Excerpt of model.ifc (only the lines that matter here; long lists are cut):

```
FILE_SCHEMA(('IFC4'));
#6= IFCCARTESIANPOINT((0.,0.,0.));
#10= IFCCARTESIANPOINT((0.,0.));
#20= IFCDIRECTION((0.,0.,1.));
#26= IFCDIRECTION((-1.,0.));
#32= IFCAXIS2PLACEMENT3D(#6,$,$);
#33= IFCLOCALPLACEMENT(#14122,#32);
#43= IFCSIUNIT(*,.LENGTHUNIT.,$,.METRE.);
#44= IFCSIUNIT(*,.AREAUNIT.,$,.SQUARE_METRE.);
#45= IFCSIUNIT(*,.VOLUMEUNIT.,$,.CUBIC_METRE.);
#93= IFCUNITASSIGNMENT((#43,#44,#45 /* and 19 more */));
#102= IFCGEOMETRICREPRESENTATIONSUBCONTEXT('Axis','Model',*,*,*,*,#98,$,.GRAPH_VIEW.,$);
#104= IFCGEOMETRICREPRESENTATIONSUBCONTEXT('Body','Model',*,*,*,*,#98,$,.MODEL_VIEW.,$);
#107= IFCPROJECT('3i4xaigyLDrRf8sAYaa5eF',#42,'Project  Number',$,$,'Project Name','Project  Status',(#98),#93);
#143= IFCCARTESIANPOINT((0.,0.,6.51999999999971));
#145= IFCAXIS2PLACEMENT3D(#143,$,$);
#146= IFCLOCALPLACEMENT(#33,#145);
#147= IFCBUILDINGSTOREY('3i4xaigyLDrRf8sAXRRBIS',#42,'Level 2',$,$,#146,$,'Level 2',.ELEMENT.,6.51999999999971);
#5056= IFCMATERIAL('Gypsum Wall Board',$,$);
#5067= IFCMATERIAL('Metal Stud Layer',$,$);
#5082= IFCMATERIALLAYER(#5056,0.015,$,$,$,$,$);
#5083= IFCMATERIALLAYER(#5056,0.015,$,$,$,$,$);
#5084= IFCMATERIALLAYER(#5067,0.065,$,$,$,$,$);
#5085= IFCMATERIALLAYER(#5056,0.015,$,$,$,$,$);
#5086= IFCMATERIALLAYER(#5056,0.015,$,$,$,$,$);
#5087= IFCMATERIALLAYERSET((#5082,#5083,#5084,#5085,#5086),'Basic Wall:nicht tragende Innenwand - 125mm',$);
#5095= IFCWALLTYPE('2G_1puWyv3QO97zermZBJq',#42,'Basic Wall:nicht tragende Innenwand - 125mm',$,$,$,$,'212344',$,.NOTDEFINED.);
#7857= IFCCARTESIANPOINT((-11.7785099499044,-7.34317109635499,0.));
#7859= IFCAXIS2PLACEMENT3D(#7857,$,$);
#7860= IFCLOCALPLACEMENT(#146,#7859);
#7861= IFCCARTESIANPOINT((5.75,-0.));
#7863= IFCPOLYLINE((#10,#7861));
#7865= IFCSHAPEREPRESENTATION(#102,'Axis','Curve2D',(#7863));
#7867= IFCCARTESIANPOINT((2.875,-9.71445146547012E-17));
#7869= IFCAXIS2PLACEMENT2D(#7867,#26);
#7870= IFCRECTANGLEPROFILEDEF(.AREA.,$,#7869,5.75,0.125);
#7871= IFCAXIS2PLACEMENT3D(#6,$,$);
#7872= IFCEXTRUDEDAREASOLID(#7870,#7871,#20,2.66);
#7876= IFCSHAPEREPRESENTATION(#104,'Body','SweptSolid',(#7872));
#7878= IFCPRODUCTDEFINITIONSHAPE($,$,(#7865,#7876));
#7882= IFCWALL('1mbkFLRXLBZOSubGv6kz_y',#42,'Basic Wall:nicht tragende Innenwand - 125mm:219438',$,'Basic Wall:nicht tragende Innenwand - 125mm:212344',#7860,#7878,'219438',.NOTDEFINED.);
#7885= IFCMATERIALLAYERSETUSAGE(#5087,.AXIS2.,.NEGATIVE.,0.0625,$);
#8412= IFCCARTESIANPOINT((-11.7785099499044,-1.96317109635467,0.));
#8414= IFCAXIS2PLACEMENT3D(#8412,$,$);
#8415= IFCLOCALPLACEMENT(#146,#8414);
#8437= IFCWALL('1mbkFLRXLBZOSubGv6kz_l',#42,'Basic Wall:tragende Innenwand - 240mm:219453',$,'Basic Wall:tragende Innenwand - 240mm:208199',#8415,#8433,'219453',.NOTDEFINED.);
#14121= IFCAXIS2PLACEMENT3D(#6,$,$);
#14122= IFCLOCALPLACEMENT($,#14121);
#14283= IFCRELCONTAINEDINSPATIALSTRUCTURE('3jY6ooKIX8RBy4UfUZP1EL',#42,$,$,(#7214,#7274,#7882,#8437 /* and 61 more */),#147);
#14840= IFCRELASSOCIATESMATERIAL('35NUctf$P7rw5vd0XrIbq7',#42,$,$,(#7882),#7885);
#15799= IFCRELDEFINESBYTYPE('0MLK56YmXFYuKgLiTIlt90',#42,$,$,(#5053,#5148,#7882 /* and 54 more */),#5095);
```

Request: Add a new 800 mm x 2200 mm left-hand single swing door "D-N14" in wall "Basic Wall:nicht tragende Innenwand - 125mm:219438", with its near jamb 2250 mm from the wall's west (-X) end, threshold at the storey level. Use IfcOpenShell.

```python
import numpy as np
import ifcopenshell
import ifcopenshell.api.feature
import ifcopenshell.api.geometry
import ifcopenshell.api.root
import ifcopenshell.api.spatial
import ifcopenshell.geom
import ifcopenshell.util.element
import ifcopenshell.util.placement
import ifcopenshell.util.representation
import ifcopenshell.util.shape
import ifcopenshell.util.unit

model = ifcopenshell.open("model.ifc")
unit_scale = ifcopenshell.util.unit.calculate_unit_scale(model)
settings = ifcopenshell.geom.settings()


def volume(element):
    """Net volume in cubic metres, openings subtracted."""
    shape = ifcopenshell.geom.create_shape(settings, element)
    return ifcopenshell.util.shape.get_volume(shape.geometry)


wall = model.by_guid("1mbkFLRXLBZOSubGv6kz_y")
storey = ifcopenshell.util.element.get_container(wall, ifc_class="IfcBuildingStorey")
context = ifcopenshell.util.representation.get_context(model, "Model", "Body", "MODEL_VIEW")
before = volume(wall)

width, height, from_end, sill = 0.8, 2.2, 2.25, 0.0  # metres

# The wall runs along its own X axis, and the end named is its -X end.
wall_shape = ifcopenshell.geom.create_shape(settings, wall)
x, y, z = ifcopenshell.util.shape.get_vertices(wall_shape.geometry).T
start = x.min() + from_end
face, thickness = float(y.min()), float(y.max() - y.min())
wall_matrix = ifcopenshell.util.placement.get_local_placement(wall.ObjectPlacement)
level = ifcopenshell.util.placement.get_local_placement(storey.ObjectPlacement)[2, 3]


def in_wall(x, y):
    """Placement at x, y metres in the wall's axes, at sill height."""
    matrix = wall_matrix.copy()
    matrix[:, 3] = wall_matrix @ np.array([x / unit_scale, y / unit_scale, 0.0, 1.0])
    matrix[2, 3] = level + sill / unit_scale
    return matrix


# Opening: a box that overshoots both wall faces by 50 mm.
opening = ifcopenshell.api.root.create_entity(model, ifc_class="IfcOpeningElement", predefined_type="OPENING")
box = ifcopenshell.api.geometry.add_wall_representation(
    model, context=context, length=width, height=height, thickness=thickness + 0.1
)
ifcopenshell.api.geometry.assign_representation(model, product=opening, representation=box)
ifcopenshell.api.geometry.edit_object_placement(model, product=opening, matrix=in_wall(start, face - 0.05), is_si=False)
ifcopenshell.api.feature.add_feature(model, feature=opening, element=wall)

door = ifcopenshell.api.root.create_entity(model, ifc_class="IfcDoor", name="D-N14", predefined_type="DOOR")
door.OverallWidth, door.OverallHeight = width / unit_scale, height / unit_scale
door.OperationType = "SINGLE_SWING_LEFT"
body = ifcopenshell.api.geometry.add_door_representation(
    model,
    context=context,
    overall_width=door.OverallWidth,
    overall_height=door.OverallHeight,
    operation_type="SINGLE_SWING_LEFT",
    lining_properties={"LiningDepth": thickness / unit_scale, "ThresholdDepth": thickness / unit_scale},
)
ifcopenshell.api.geometry.assign_representation(model, product=door, representation=body)
ifcopenshell.api.spatial.assign_container(model, products=[door], relating_structure=storey)
ifcopenshell.api.feature.add_filling(model, opening=opening, element=door)

# The lining spans the wall, so the door starts at the wall face.
ifcopenshell.api.geometry.edit_object_placement(model, product=door, matrix=in_wall(start, face), is_si=False)

after = volume(wall)

print(f"wall volume {before:.3f} -> {after:.3f} m3")

model.write("model_v2.ifc")
```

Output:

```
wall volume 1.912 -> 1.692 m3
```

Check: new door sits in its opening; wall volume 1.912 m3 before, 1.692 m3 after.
